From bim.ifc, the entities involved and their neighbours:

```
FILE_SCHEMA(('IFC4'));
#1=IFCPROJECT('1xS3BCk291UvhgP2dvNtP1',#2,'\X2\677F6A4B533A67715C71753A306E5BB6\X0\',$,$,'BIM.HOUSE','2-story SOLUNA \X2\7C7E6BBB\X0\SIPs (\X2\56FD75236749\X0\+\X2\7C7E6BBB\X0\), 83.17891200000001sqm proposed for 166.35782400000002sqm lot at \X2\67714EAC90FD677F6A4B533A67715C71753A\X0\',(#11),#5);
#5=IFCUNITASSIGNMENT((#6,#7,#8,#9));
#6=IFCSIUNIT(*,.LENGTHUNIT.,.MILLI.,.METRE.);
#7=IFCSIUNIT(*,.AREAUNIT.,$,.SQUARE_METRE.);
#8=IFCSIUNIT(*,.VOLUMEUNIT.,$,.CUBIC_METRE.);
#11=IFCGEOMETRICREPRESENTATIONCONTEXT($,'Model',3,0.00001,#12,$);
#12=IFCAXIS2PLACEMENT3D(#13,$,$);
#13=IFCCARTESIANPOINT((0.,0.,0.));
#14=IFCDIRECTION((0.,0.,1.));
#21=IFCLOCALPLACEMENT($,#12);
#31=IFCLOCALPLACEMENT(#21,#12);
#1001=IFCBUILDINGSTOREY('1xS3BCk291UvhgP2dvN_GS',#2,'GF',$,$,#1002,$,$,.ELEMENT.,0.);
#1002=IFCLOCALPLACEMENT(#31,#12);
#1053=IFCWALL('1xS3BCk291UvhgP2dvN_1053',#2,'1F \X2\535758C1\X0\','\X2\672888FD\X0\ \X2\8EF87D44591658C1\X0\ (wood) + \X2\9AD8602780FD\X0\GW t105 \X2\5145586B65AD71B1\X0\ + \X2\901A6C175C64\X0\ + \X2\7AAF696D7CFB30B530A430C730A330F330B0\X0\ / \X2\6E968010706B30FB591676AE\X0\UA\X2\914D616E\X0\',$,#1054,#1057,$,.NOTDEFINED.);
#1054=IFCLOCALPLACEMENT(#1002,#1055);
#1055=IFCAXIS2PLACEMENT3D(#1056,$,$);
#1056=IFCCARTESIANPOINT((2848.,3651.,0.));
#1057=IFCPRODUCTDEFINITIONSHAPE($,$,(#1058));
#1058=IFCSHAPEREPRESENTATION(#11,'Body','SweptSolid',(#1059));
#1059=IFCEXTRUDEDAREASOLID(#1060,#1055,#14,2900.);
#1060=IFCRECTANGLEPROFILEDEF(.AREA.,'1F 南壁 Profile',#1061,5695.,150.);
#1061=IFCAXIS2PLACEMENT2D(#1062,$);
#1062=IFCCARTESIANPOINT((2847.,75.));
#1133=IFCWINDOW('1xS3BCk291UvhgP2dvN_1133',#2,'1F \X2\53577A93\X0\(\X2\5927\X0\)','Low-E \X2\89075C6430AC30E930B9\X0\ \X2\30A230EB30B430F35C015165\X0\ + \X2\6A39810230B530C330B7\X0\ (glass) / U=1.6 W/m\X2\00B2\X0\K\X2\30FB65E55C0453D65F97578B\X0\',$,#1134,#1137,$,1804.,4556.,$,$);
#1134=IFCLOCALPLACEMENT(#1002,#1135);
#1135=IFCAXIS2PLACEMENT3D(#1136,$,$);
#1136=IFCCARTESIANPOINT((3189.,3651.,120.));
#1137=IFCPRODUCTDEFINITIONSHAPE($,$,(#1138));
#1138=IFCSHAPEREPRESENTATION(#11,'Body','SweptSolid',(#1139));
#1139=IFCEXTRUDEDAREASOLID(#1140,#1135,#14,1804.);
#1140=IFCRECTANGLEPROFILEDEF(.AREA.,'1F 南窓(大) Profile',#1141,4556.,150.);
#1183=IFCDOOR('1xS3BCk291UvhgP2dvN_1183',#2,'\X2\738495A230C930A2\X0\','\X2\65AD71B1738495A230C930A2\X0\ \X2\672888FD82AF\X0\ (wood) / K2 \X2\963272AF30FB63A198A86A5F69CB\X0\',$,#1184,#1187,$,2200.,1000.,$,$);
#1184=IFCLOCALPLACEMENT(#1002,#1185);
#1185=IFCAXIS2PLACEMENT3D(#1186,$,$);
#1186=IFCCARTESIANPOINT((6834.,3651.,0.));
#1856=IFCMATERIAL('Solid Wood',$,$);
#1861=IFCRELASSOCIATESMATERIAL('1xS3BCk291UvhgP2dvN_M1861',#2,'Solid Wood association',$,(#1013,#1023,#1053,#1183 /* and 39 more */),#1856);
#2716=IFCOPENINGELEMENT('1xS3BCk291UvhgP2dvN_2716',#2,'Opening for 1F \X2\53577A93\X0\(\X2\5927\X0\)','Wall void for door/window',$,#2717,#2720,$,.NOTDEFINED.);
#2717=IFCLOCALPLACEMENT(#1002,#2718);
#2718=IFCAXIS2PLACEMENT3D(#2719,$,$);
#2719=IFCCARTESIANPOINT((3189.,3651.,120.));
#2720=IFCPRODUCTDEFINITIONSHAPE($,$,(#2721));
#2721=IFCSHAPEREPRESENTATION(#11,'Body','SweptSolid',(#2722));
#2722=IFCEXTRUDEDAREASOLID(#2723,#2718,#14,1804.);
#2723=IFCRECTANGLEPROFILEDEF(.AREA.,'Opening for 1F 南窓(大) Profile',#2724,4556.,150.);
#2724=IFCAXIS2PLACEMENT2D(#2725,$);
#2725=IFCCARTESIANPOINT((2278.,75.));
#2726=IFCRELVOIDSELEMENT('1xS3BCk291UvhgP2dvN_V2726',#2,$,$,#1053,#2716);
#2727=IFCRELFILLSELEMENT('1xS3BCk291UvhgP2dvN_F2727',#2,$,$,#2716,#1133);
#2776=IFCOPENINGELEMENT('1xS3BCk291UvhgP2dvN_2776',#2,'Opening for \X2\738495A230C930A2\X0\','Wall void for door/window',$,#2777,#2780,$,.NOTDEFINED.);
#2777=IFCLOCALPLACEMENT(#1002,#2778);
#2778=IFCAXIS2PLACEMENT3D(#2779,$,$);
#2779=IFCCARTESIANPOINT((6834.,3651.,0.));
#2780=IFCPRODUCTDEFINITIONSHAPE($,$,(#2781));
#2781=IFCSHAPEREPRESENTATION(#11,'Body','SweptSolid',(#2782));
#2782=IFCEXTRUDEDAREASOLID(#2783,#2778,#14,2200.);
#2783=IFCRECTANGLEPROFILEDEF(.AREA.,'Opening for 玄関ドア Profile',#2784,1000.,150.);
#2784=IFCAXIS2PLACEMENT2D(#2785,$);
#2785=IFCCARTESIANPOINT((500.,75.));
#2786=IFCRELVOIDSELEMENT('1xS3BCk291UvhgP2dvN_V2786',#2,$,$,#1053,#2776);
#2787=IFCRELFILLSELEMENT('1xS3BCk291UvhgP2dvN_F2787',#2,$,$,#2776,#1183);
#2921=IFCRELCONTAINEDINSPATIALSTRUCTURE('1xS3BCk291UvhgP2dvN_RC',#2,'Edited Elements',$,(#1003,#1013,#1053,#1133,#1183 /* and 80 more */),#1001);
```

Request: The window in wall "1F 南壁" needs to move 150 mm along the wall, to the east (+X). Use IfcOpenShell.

```python
import ifcopenshell
import ifcopenshell.api.geometry
import ifcopenshell.util.placement

model = ifcopenshell.open("bim.ifc")

window = model.by_id(1133)
opening = window.FillsVoids[0].RelatingOpeningElement
wall = opening.VoidsElements[0].RelatingBuildingElement

wall_matrix = ifcopenshell.util.placement.get_local_placement(wall.ObjectPlacement)
shift = wall_matrix[:3, 0] * 150.0
before = ifcopenshell.util.placement.get_local_placement(window.ObjectPlacement)[:3, 3].copy()

# The window is not placed relative to its opening, so move both.
for product in (opening, window):
    matrix = ifcopenshell.util.placement.get_local_placement(product.ObjectPlacement)
    matrix[:3, 3] += shift
    ifcopenshell.api.geometry.edit_object_placement(model, product=product, matrix=matrix, is_si=False)

after = ifcopenshell.util.placement.get_local_placement(window.ObjectPlacement)[:3, 3]
print("window moved by", (after - before).round(3) + 0.0)

model.write("bim_v2.ifc")
```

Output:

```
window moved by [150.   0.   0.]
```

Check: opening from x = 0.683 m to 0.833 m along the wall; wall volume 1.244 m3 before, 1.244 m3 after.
